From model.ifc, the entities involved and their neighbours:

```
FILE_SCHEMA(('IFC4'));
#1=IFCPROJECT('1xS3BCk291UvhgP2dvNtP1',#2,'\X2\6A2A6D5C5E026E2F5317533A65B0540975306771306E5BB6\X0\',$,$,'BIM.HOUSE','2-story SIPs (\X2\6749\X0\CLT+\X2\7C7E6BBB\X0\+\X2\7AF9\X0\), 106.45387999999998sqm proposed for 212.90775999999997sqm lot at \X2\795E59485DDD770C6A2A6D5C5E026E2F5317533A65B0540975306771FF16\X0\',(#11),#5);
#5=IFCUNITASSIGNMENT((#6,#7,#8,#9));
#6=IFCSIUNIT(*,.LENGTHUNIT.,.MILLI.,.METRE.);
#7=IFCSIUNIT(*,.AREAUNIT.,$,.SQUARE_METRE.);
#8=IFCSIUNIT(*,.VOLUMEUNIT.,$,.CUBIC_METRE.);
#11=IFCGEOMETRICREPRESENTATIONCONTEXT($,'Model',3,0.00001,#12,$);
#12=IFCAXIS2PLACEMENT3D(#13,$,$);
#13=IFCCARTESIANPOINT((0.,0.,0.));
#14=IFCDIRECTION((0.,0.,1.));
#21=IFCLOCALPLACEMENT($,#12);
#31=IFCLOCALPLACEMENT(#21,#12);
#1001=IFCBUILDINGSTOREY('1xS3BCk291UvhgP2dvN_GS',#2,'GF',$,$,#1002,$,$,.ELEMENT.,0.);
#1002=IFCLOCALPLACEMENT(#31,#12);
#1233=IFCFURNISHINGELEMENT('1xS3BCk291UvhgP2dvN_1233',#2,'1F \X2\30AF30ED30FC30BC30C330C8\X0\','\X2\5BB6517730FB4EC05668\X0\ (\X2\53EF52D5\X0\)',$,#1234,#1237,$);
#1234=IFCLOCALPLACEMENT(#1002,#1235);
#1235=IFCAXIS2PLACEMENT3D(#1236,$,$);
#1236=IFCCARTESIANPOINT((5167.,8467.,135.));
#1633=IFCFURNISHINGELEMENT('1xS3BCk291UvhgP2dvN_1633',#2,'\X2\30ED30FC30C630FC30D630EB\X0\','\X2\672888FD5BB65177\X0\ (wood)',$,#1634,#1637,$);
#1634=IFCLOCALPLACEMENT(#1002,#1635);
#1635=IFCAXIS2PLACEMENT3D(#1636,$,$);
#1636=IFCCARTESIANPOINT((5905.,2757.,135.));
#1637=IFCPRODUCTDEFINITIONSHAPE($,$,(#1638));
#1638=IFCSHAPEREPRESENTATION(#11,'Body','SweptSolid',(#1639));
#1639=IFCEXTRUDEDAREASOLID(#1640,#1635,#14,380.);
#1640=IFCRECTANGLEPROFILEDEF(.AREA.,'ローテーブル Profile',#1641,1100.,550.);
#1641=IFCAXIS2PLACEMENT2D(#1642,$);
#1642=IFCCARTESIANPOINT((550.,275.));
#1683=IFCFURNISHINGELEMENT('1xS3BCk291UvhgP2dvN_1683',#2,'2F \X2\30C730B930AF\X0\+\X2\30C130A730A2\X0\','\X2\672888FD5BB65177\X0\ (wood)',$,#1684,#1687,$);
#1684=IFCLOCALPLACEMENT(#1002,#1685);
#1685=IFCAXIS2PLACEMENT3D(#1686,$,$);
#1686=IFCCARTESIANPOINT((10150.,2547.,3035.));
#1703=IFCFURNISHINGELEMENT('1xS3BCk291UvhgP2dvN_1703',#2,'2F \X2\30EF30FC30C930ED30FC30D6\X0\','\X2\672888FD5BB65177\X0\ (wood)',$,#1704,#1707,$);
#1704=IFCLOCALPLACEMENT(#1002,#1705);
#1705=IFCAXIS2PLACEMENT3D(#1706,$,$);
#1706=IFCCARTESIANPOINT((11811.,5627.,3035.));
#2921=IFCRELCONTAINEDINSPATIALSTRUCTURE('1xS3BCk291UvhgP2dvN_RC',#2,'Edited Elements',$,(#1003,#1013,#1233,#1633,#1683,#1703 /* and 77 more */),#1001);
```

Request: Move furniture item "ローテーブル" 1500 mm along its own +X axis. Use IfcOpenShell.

```python
import ifcopenshell
import ifcopenshell.api.geometry
import ifcopenshell.util.placement

model = ifcopenshell.open("model.ifc")

item = model.by_guid("1xS3BCk291UvhgP2dvN_1633")
matrix = ifcopenshell.util.placement.get_local_placement(item.ObjectPlacement)
matrix[:3, 3] += matrix[:3, 0] * 1500.0
ifcopenshell.api.geometry.edit_object_placement(model, product=item, matrix=matrix, is_si=False)

print(ifcopenshell.util.placement.get_local_placement(item.ObjectPlacement).round(3) + 0.0)

model.write("model-out.ifc")
```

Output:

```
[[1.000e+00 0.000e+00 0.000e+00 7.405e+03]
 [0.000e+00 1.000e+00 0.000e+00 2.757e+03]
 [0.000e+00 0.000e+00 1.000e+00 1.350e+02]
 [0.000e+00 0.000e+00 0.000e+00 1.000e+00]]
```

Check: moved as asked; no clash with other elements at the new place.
